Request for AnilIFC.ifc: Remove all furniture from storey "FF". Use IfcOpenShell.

First a look at what the model holds.

```python
import ifcopenshell
import ifcopenshell.util.element

model = ifcopenshell.open("AnilIFC.ifc")
print(model.schema)
storey = next(s for s in model.by_type("IfcBuildingStorey") if s.Name == "FF")
furniture = [e for e in ifcopenshell.util.element.get_decomposition(storey) if e.is_a("IfcFurnishingElement")]
seen = {}
for e in furniture:
    element_type = ifcopenshell.util.element.get_type(e)
    name = element_type.Name if element_type not in (None, e) else None
    seen[name] = seen.get(name, 0) + 1
for name, count in sorted(seen.items(), key=str):
    print(count, "x", name)
```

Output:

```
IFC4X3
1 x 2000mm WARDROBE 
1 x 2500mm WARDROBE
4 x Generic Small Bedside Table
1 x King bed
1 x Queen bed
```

```python
import ifcopenshell
import ifcopenshell.api.root
import ifcopenshell.util.element

model = ifcopenshell.open("AnilIFC.ifc")

storey = next(s for s in model.by_type("IfcBuildingStorey") if s.Name == "FF")
furniture = [e for e in ifcopenshell.util.element.get_decomposition(storey) if e.is_a("IfcFurnishingElement")]

for e in furniture:
    ifcopenshell.api.root.remove_product(model, product=e)
print(len(furniture), "removed")

model.write("AnilIFC_rev.ifc")
```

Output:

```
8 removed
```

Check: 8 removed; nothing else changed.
